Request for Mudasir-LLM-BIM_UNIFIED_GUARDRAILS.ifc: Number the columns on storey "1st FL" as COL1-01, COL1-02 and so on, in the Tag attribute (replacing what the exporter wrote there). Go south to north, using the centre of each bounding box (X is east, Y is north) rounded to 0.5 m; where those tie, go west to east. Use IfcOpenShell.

First a look at what the model holds.

```python
import ifcopenshell
import ifcopenshell.util.element
import ifcopenshell.util.placement

model = ifcopenshell.open("Mudasir-LLM-BIM_UNIFIED_GUARDRAILS.ifc")
print(model.schema)
storey = next(s for s in model.by_type("IfcBuildingStorey") if s.Name == "1st FL")
columns = [e for e in ifcopenshell.util.element.get_decomposition(storey) if e.is_a("IfcColumn")]
for e in sorted(columns, key=lambda e: e.id()):
    origin = ifcopenshell.util.placement.get_local_placement(e.ObjectPlacement)[:3, 3]
    print(e.id(), e.Tag, e.Name, origin.round(2) + 0.0, sep=" | ")
```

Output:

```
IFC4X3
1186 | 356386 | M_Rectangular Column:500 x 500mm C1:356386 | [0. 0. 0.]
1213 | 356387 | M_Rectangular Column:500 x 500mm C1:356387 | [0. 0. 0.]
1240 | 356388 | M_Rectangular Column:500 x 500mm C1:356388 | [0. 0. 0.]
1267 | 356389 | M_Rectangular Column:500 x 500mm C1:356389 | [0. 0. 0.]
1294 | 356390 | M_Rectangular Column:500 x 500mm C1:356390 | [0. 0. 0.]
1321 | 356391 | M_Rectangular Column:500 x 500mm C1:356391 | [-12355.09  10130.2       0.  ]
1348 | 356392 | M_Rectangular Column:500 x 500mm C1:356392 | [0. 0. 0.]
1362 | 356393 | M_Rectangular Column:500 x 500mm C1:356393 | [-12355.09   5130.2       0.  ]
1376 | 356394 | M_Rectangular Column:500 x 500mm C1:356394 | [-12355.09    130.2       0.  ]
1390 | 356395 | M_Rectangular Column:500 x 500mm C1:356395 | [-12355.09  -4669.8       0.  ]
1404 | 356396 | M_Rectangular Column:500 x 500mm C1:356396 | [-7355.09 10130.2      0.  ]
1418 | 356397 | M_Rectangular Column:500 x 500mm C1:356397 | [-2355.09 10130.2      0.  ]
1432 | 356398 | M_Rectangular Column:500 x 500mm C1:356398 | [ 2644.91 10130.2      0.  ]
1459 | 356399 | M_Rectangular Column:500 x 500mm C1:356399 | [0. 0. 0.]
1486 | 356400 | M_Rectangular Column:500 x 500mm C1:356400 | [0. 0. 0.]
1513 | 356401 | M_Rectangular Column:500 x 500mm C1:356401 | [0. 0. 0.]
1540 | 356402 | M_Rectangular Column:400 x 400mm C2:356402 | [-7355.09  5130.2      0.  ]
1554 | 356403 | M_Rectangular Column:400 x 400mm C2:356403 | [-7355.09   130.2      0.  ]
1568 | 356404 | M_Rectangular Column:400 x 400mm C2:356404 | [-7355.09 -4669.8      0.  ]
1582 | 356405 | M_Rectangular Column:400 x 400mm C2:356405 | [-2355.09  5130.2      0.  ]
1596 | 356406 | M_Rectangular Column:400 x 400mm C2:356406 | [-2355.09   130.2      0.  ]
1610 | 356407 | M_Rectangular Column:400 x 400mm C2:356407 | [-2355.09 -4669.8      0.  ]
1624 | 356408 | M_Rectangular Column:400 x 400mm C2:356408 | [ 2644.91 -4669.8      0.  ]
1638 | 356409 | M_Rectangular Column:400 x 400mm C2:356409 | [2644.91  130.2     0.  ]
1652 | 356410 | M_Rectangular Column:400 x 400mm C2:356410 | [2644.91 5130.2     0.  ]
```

```python
import ifcopenshell
import ifcopenshell.geom
import ifcopenshell.util.element
import ifcopenshell.util.shape

model = ifcopenshell.open("Mudasir-LLM-BIM_UNIFIED_GUARDRAILS.ifc")
settings = ifcopenshell.geom.settings()
settings.set("use-world-coords", True)


def centre(element):
    shape = ifcopenshell.geom.create_shape(settings, element)
    return ifcopenshell.util.shape.get_bbox_centroid(shape.geometry)


storey = next(s for s in model.by_type("IfcBuildingStorey") if s.Name == "1st FL")
columns = [e for e in ifcopenshell.util.element.get_decomposition(storey) if e.is_a("IfcColumn")]

# Insertion points can sit at a corner or the storey origin, so sort by the geometry (in metres).
centres = {e: centre(e) for e in columns}
columns.sort(key=lambda e: (round(centres[e][1] / 0.5), centres[e][0]))

for i, e in enumerate(columns, start=1):
    number = f"COL1-{i:02d}"
    e.Tag = number
    print(e.id(), number)

model.write("Mudasir-LLM-BIM_UNIFIED_GUARDRAILS_updated.ifc")
```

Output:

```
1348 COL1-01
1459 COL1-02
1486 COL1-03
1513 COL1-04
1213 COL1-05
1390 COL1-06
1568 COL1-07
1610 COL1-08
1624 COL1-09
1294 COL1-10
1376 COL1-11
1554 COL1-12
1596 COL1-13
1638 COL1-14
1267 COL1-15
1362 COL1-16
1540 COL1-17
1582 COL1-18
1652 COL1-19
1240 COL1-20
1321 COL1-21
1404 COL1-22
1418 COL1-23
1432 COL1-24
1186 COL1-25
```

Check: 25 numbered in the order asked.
